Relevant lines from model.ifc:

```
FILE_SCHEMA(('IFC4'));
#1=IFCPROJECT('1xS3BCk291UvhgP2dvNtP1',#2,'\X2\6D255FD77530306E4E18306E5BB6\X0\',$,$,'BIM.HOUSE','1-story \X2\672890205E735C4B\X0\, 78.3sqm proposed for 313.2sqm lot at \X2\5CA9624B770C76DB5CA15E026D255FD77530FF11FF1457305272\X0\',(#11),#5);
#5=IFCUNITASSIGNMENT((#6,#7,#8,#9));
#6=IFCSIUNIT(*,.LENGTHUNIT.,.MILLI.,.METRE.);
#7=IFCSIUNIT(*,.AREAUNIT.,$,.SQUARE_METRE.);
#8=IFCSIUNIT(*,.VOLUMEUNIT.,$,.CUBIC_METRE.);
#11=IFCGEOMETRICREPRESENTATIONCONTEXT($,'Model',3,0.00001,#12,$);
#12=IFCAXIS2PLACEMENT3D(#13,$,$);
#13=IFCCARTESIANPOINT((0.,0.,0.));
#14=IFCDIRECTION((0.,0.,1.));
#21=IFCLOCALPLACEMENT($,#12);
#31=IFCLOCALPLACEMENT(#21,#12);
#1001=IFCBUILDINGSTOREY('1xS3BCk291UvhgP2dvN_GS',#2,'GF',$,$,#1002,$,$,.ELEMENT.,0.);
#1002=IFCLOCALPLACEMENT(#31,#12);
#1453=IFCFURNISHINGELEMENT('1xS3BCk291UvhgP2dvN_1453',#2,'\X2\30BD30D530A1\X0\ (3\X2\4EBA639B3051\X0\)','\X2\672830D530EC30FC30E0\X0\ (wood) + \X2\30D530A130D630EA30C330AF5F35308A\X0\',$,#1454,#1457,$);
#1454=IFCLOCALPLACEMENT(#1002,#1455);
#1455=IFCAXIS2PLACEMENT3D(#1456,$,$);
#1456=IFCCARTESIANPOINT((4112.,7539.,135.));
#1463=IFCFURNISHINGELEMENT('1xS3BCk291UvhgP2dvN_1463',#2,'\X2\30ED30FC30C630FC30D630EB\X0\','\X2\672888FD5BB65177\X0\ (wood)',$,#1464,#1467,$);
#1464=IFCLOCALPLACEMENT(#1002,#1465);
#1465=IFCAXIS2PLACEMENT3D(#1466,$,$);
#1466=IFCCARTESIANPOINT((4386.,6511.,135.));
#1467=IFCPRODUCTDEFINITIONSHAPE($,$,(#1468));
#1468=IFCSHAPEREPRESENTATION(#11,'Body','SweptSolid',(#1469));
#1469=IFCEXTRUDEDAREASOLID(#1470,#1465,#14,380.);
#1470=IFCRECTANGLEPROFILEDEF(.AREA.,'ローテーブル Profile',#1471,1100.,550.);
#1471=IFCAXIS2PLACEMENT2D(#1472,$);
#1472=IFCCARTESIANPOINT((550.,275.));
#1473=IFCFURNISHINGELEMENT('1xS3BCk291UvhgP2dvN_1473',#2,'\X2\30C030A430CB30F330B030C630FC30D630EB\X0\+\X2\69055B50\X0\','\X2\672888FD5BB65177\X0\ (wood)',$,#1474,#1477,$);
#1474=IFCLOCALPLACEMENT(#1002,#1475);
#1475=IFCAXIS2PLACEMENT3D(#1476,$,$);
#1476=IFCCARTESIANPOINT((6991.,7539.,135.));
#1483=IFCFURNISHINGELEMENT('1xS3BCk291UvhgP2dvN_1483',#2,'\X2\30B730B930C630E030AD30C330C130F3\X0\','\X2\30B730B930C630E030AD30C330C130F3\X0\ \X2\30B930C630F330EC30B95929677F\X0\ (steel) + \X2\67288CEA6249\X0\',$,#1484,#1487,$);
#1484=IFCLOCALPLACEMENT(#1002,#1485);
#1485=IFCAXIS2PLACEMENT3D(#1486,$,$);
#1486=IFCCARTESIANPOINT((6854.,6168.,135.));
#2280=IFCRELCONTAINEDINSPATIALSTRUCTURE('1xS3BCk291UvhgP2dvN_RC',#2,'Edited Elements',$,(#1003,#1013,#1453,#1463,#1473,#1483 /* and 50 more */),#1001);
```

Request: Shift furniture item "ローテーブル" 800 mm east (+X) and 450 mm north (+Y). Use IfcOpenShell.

```python
import ifcopenshell
import ifcopenshell.api.geometry
import ifcopenshell.util.placement
import ifcopenshell.util.unit

model = ifcopenshell.open("model.ifc")
unit_scale = ifcopenshell.util.unit.calculate_unit_scale(model)

item = model.by_guid("1xS3BCk291UvhgP2dvN_1463")
matrix = ifcopenshell.util.placement.get_local_placement(item.ObjectPlacement)
matrix[0, 3] += 0.8 / unit_scale
matrix[1, 3] += 0.45 / unit_scale
ifcopenshell.api.geometry.edit_object_placement(model, product=item, matrix=matrix, is_si=False)

print(ifcopenshell.util.placement.get_local_placement(item.ObjectPlacement).round(3) + 0.0)

model.write("model-out.ifc")
```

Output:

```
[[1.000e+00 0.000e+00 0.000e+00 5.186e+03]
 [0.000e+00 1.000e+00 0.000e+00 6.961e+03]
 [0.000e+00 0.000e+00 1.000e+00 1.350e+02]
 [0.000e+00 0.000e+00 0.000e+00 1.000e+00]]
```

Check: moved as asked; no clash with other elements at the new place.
